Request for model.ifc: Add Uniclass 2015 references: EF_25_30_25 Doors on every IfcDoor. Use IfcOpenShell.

First a look at what the model holds.

```python
import ifcopenshell

model = ifcopenshell.open("model.ifc")
print(model.schema)
print("classifications:", [c.Name for c in model.by_type("IfcClassification")])
for ifc_class in ("IfcDoor", "IfcRoof", "IfcStair", "IfcWall", "IfcWindow"):
    print(ifc_class, len(model.by_type(ifc_class)))
```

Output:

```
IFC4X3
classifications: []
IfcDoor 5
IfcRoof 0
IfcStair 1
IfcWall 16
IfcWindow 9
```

```python
import ifcopenshell
import ifcopenshell.api.classification

model = ifcopenshell.open("model.ifc")

system = ifcopenshell.api.classification.add_classification(model, classification="Uniclass 2015")

codes = {
    "IfcDoor": ("EF_25_30_25", "Doors"),
}
for ifc_class, (code, name) in codes.items():
    products = model.by_type(ifc_class)
    ifcopenshell.api.classification.add_reference(
        model, products=products, classification=system, identification=code, name=name
    )
    print(code, len(products))

model.write("model_updated.ifc")
```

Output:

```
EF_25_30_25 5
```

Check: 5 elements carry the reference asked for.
